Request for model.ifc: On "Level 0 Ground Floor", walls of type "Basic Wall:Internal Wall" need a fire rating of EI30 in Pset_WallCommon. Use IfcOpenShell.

First a look at what the model holds.

```python
import ifcopenshell
import ifcopenshell.util.element

model = ifcopenshell.open("model.ifc")
print(model.schema)
storey = next(s for s in model.by_type("IfcBuildingStorey") if s.Name == "Level 0 Ground Floor")
walls = [e for e in ifcopenshell.util.element.get_decomposition(storey) if e.is_a("IfcWall")]
seen = {}
for e in walls:
    element_type = ifcopenshell.util.element.get_type(e)
    key = (element_type.Name if element_type != e and element_type else None, ifcopenshell.util.element.get_pset(e, "Pset_WallCommon", "FireRating"))
    seen[key] = seen.get(key, 0) + 1
for (name, value), count in sorted(seen.items(), key=str):
    print(count, "x", name, "|", value)
```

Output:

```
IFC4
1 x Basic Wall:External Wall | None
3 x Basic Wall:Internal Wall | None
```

```python
import ifcopenshell
import ifcopenshell.api.pset
import ifcopenshell.util.element

model = ifcopenshell.open("model.ifc")

storey = next(s for s in model.by_type("IfcBuildingStorey") if s.Name == "Level 0 Ground Floor")
walls = [e for e in ifcopenshell.util.element.get_decomposition(storey) if e.is_a("IfcWall")]

count = 0
for e in walls:
    element_type = ifcopenshell.util.element.get_type(e)
    if element_type in (None, e) or element_type.Name != "Basic Wall:Internal Wall":
        continue
    # add_pset returns the element's existing set when there is one.
    pset = ifcopenshell.api.pset.add_pset(model, product=e, name="Pset_WallCommon")
    ifcopenshell.api.pset.edit_pset(model, pset=pset, properties={"FireRating": "EI30"})
    count += 1

print(count, "walls updated")

model.write("model-out.ifc")
```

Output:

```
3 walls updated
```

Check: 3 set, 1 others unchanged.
